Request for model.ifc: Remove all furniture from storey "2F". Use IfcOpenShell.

First a look at what the model holds.

```python
import ifcopenshell
import ifcopenshell.util.element

model = ifcopenshell.open("model.ifc")
print(model.schema)
storey = next(s for s in model.by_type("IfcBuildingStorey") if s.Name == "2F")
furniture = [e for e in ifcopenshell.util.element.get_decomposition(storey) if e.is_a("IfcFurnishingElement")]
seen = {}
for e in furniture:
    element_type = ifcopenshell.util.element.get_type(e)
    name = element_type.Name if element_type not in (None, e) else None
    seen[name] = seen.get(name, 0) + 1
for name, count in sorted(seen.items(), key=str):
    print(count, "x", name)
```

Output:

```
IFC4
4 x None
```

```python
import ifcopenshell
import ifcopenshell.api.root
import ifcopenshell.util.element

model = ifcopenshell.open("model.ifc")

storey = next(s for s in model.by_type("IfcBuildingStorey") if s.Name == "2F")
furniture = [e for e in ifcopenshell.util.element.get_decomposition(storey) if e.is_a("IfcFurnishingElement")]

for e in furniture:
    ifcopenshell.api.root.remove_product(model, product=e)
print(len(furniture), "removed")

model.write("model_rev.ifc")
```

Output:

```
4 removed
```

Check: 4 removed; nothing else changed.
